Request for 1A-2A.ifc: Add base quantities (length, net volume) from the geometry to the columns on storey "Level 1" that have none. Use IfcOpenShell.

First a look at what the model holds.

```python
import ifcopenshell
import ifcopenshell.util.element
import ifcopenshell.util.unit

model = ifcopenshell.open("1A-2A.ifc")
print(model.schema)
for unit_type in ("LENGTHUNIT", "AREAUNIT", "VOLUMEUNIT"):
    print(unit_type, ifcopenshell.util.unit.calculate_unit_scale(model, unit_type))
storey = next(s for s in model.by_type("IfcBuildingStorey") if s.Name == "Level 1")
columns = [e for e in ifcopenshell.util.element.get_decomposition(storey) if e.is_a("IfcColumn")]
for e in sorted(columns, key=lambda e: e.id()):
    print(e.id(), e.is_a(), e.Name, list(ifcopenshell.util.element.get_psets(e, qtos_only=True)), sep=" | ")
```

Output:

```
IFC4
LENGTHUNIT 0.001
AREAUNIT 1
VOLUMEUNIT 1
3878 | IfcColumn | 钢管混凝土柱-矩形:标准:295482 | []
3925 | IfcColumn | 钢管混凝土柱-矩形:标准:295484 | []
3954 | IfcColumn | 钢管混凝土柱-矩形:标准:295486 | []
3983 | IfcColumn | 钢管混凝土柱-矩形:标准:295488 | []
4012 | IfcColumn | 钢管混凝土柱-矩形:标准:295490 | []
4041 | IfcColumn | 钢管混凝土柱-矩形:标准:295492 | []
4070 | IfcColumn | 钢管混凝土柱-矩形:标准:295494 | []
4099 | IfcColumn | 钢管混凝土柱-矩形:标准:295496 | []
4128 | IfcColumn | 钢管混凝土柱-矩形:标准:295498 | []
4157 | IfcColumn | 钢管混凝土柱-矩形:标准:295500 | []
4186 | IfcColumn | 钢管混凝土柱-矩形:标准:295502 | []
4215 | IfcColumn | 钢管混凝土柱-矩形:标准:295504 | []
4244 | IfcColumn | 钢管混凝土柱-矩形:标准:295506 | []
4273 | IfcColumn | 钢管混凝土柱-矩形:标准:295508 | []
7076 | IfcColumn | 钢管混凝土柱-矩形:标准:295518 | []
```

```python
import ifcopenshell
import ifcopenshell.api.pset
import ifcopenshell.geom
import ifcopenshell.util.element
import ifcopenshell.util.shape
import ifcopenshell.util.unit

model = ifcopenshell.open("1A-2A.ifc")
unit_scale = ifcopenshell.util.unit.calculate_unit_scale(model)
volume_scale = ifcopenshell.util.unit.calculate_unit_scale(model, "VOLUMEUNIT")
settings = ifcopenshell.geom.settings()

storey = next(s for s in model.by_type("IfcBuildingStorey") if s.Name == "Level 1")
columns = [e for e in ifcopenshell.util.element.get_decomposition(storey) if e.is_a("IfcColumn")]

for e in sorted(columns, key=lambda e: e.id()):
    if ifcopenshell.util.element.get_psets(e, qtos_only=True, should_inherit=False):
        continue
    # Geometry comes back in metres, in the element's own axes.
    shape = ifcopenshell.geom.create_shape(settings, e)
    values = {
        "Length": ifcopenshell.util.shape.get_z(shape.geometry) / unit_scale,
        "NetVolume": ifcopenshell.util.shape.get_volume(shape.geometry) / volume_scale,
    }
    qto = ifcopenshell.api.pset.add_qto(model, product=e, name="Qto_ColumnBaseQuantities")
    ifcopenshell.api.pset.edit_qto(model, qto=qto, properties=values)
    print(e.id(), {k: round(v, 3) for k, v in values.items()})

model.write("1A-2A_edited.ifc")
```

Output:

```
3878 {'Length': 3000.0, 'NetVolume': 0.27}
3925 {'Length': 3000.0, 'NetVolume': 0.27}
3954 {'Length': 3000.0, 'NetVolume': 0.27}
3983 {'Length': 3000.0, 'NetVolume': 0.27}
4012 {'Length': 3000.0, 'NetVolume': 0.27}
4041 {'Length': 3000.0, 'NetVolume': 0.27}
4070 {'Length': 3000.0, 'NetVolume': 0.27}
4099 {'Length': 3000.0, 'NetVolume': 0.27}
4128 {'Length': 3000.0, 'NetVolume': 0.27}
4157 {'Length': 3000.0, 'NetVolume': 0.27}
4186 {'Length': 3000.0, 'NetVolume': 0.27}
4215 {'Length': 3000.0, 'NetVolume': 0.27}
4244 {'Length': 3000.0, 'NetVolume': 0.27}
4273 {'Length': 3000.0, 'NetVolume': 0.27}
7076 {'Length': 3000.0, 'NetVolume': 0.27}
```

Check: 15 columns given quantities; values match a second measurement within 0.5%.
